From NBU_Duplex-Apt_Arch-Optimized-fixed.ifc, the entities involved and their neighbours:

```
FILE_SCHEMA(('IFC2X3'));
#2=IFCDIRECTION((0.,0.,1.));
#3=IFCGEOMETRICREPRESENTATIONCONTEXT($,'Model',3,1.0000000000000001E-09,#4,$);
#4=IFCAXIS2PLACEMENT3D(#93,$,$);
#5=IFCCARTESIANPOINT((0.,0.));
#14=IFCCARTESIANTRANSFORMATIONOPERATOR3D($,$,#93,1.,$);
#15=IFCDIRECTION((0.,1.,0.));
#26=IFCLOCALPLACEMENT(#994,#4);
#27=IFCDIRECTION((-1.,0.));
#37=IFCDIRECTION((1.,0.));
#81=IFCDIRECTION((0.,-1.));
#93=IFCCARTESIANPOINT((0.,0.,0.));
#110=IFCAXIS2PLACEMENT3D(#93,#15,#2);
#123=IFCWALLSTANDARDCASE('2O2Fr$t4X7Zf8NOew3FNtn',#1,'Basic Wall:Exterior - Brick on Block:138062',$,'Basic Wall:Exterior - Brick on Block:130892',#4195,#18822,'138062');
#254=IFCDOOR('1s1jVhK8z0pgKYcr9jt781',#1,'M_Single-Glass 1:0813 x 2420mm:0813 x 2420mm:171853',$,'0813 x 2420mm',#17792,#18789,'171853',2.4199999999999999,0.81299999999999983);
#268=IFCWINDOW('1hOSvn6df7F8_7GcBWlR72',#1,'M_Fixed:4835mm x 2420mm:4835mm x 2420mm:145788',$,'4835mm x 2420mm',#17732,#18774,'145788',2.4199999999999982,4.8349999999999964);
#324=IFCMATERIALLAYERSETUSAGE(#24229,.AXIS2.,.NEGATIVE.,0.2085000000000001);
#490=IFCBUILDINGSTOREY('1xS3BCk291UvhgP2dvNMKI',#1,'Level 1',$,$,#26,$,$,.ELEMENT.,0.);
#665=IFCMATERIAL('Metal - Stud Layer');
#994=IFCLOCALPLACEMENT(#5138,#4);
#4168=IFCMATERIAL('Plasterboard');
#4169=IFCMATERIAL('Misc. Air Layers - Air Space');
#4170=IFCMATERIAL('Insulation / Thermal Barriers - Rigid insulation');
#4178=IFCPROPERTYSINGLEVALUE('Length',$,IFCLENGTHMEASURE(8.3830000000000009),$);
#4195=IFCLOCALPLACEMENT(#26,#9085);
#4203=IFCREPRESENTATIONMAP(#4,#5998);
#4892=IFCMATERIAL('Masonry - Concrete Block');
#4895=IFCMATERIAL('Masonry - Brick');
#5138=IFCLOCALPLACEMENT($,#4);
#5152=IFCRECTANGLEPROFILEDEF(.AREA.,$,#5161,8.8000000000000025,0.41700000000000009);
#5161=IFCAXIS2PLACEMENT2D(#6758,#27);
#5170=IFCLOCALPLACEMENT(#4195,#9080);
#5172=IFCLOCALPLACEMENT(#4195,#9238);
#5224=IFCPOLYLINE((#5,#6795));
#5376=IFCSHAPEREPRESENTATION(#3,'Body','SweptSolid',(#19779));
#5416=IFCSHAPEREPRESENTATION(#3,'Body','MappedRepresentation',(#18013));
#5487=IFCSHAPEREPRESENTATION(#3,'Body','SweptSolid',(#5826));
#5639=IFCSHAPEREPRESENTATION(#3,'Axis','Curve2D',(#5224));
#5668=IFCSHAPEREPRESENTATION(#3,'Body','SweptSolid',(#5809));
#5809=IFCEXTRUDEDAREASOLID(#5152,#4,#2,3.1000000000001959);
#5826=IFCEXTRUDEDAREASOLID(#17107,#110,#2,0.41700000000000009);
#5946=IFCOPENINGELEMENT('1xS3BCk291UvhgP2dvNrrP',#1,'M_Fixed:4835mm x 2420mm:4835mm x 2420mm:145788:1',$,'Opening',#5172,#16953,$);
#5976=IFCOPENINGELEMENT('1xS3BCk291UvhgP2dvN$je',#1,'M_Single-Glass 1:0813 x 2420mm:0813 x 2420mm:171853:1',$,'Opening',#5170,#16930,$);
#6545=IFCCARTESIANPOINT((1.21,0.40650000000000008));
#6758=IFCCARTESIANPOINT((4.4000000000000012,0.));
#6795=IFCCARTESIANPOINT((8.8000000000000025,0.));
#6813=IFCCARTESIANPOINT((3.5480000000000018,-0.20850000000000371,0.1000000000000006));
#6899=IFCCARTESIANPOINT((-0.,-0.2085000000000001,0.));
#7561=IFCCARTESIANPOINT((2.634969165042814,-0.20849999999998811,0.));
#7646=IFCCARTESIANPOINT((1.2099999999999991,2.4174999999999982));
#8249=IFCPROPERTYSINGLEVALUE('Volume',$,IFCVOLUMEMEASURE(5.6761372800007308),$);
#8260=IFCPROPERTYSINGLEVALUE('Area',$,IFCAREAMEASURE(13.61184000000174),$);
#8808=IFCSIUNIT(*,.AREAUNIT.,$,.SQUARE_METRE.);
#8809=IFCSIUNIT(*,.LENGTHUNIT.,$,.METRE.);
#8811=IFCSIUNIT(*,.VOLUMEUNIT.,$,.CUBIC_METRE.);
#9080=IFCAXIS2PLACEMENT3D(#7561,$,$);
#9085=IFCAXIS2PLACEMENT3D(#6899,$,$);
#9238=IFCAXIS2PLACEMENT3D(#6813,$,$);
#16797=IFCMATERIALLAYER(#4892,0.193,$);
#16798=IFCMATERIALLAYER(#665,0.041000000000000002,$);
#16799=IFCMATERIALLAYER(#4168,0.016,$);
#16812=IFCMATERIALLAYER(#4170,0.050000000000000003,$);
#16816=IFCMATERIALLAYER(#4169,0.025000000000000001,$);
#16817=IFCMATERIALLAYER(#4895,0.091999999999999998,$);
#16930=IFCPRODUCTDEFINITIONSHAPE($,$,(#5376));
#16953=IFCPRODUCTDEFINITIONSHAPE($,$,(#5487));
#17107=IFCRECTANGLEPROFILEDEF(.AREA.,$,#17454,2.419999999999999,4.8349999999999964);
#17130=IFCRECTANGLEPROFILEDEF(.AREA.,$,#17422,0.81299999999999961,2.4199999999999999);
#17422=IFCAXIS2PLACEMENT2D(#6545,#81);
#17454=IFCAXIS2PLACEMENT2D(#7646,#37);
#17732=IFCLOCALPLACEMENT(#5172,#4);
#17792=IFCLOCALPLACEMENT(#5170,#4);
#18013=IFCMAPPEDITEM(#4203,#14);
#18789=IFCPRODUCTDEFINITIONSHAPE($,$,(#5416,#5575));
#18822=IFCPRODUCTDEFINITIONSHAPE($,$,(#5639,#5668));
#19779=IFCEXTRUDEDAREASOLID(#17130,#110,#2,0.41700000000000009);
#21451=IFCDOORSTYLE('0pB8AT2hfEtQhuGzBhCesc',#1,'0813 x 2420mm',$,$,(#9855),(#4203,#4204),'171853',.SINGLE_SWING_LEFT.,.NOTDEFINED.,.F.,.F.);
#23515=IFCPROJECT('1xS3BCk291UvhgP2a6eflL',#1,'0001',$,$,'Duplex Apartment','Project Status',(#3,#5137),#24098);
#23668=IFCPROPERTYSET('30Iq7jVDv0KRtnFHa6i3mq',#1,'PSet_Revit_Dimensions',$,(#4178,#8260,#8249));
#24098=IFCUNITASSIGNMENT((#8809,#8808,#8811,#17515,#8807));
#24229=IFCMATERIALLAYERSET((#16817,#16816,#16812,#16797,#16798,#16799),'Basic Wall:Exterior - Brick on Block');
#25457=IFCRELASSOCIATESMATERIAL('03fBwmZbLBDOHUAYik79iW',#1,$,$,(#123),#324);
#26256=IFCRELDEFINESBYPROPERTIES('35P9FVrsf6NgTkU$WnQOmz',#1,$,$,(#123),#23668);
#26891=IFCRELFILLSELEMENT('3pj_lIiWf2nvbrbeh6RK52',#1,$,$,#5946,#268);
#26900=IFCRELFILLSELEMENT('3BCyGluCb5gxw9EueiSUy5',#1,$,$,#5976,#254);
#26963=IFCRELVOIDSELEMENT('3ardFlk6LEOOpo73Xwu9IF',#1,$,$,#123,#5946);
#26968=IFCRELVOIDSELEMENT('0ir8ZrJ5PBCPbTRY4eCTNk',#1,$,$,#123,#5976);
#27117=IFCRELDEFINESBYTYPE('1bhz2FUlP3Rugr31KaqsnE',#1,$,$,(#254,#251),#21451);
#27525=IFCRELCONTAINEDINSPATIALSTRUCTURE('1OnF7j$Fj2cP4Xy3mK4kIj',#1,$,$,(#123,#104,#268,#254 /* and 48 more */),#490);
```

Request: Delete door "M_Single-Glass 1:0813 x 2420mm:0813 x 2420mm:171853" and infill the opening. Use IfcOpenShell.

```python
import ifcopenshell
import ifcopenshell.api.feature
import ifcopenshell.api.pset
import ifcopenshell.api.root
import ifcopenshell.geom
import ifcopenshell.util.element
import ifcopenshell.util.shape
import ifcopenshell.util.unit

model = ifcopenshell.open("NBU_Duplex-Apt_Arch-Optimized-fixed.ifc")
area_scale = ifcopenshell.util.unit.calculate_unit_scale(model, "AREAUNIT")
volume_scale = ifcopenshell.util.unit.calculate_unit_scale(model, "VOLUMEUNIT")
settings = ifcopenshell.geom.settings()


def volume(element):
    """Net volume in cubic metres, openings subtracted."""
    shape = ifcopenshell.geom.create_shape(settings, element)
    return ifcopenshell.util.shape.get_volume(shape.geometry)


door = model.by_guid("1s1jVhK8z0pgKYcr9jt781")
opening = door.FillsVoids[0].RelatingOpeningElement
wall = opening.VoidsElements[0].RelatingBuildingElement
before = volume(wall)

ifcopenshell.api.root.remove_product(model, product=door)
ifcopenshell.api.feature.remove_feature(model, feature=opening)

after = volume(wall)
thickness = 0.417  # wall thickness in metres

# Update the wall's stored quantities.
pset = model.by_id(ifcopenshell.util.element.get_pset(wall, "PSet_Revit_Dimensions", should_inherit=False)["id"])
ifcopenshell.api.pset.edit_pset(model, pset=pset, properties={
    "Area": model.create_entity("IfcAreaMeasure", after / thickness / area_scale),
    "Volume": model.create_entity("IfcVolumeMeasure", after / volume_scale),
})

print(f"wall volume {before:.3f} -> {after:.3f} m3")

model.write("NBU_Duplex-Apt_Arch-Optimized-fixed_rev.ifc")
```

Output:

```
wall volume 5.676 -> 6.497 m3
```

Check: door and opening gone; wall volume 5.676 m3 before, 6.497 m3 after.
